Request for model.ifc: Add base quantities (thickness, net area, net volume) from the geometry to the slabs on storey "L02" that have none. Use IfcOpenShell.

First a look at what the model holds.

```python
import ifcopenshell
import ifcopenshell.util.element
import ifcopenshell.util.unit

model = ifcopenshell.open("model.ifc")
print(model.schema)
for unit_type in ("LENGTHUNIT", "AREAUNIT", "VOLUMEUNIT"):
    print(unit_type, ifcopenshell.util.unit.calculate_unit_scale(model, unit_type))
storey = next(s for s in model.by_type("IfcBuildingStorey") if s.Name == "L02")
slabs = [e for e in ifcopenshell.util.element.get_decomposition(storey) if e.is_a("IfcSlab")]
for e in sorted(slabs, key=lambda e: e.id()):
    print(e.id(), e.is_a(), e.Name, list(ifcopenshell.util.element.get_psets(e, qtos_only=True)), sep=" | ")
```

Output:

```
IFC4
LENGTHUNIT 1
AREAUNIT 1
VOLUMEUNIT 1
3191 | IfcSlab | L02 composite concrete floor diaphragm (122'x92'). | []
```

```python
import ifcopenshell
import ifcopenshell.api.pset
import ifcopenshell.geom
import ifcopenshell.util.element
import ifcopenshell.util.shape
import ifcopenshell.util.unit

model = ifcopenshell.open("model.ifc")
unit_scale = ifcopenshell.util.unit.calculate_unit_scale(model)
area_scale = ifcopenshell.util.unit.calculate_unit_scale(model, "AREAUNIT")
volume_scale = ifcopenshell.util.unit.calculate_unit_scale(model, "VOLUMEUNIT")
settings = ifcopenshell.geom.settings()

storey = next(s for s in model.by_type("IfcBuildingStorey") if s.Name == "L02")
slabs = [e for e in ifcopenshell.util.element.get_decomposition(storey) if e.is_a("IfcSlab")]

for e in sorted(slabs, key=lambda e: e.id()):
    if ifcopenshell.util.element.get_psets(e, qtos_only=True, should_inherit=False):
        continue
    # Geometry comes back in metres, in the element's own axes.
    shape = ifcopenshell.geom.create_shape(settings, e)
    values = {
        "Width": ifcopenshell.util.shape.get_z(shape.geometry) / unit_scale,
        "NetArea": ifcopenshell.util.shape.get_footprint_area(shape.geometry) / area_scale,
        "NetVolume": ifcopenshell.util.shape.get_volume(shape.geometry) / volume_scale,
    }
    qto = ifcopenshell.api.pset.add_qto(model, product=e, name="Qto_SlabBaseQuantities")
    ifcopenshell.api.pset.edit_qto(model, qto=qto, properties=values)
    print(e.id(), {k: round(v, 3) for k, v in values.items()})

model.write("model_updated.ifc")
```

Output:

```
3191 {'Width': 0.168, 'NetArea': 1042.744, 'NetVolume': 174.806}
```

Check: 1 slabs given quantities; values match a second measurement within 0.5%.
